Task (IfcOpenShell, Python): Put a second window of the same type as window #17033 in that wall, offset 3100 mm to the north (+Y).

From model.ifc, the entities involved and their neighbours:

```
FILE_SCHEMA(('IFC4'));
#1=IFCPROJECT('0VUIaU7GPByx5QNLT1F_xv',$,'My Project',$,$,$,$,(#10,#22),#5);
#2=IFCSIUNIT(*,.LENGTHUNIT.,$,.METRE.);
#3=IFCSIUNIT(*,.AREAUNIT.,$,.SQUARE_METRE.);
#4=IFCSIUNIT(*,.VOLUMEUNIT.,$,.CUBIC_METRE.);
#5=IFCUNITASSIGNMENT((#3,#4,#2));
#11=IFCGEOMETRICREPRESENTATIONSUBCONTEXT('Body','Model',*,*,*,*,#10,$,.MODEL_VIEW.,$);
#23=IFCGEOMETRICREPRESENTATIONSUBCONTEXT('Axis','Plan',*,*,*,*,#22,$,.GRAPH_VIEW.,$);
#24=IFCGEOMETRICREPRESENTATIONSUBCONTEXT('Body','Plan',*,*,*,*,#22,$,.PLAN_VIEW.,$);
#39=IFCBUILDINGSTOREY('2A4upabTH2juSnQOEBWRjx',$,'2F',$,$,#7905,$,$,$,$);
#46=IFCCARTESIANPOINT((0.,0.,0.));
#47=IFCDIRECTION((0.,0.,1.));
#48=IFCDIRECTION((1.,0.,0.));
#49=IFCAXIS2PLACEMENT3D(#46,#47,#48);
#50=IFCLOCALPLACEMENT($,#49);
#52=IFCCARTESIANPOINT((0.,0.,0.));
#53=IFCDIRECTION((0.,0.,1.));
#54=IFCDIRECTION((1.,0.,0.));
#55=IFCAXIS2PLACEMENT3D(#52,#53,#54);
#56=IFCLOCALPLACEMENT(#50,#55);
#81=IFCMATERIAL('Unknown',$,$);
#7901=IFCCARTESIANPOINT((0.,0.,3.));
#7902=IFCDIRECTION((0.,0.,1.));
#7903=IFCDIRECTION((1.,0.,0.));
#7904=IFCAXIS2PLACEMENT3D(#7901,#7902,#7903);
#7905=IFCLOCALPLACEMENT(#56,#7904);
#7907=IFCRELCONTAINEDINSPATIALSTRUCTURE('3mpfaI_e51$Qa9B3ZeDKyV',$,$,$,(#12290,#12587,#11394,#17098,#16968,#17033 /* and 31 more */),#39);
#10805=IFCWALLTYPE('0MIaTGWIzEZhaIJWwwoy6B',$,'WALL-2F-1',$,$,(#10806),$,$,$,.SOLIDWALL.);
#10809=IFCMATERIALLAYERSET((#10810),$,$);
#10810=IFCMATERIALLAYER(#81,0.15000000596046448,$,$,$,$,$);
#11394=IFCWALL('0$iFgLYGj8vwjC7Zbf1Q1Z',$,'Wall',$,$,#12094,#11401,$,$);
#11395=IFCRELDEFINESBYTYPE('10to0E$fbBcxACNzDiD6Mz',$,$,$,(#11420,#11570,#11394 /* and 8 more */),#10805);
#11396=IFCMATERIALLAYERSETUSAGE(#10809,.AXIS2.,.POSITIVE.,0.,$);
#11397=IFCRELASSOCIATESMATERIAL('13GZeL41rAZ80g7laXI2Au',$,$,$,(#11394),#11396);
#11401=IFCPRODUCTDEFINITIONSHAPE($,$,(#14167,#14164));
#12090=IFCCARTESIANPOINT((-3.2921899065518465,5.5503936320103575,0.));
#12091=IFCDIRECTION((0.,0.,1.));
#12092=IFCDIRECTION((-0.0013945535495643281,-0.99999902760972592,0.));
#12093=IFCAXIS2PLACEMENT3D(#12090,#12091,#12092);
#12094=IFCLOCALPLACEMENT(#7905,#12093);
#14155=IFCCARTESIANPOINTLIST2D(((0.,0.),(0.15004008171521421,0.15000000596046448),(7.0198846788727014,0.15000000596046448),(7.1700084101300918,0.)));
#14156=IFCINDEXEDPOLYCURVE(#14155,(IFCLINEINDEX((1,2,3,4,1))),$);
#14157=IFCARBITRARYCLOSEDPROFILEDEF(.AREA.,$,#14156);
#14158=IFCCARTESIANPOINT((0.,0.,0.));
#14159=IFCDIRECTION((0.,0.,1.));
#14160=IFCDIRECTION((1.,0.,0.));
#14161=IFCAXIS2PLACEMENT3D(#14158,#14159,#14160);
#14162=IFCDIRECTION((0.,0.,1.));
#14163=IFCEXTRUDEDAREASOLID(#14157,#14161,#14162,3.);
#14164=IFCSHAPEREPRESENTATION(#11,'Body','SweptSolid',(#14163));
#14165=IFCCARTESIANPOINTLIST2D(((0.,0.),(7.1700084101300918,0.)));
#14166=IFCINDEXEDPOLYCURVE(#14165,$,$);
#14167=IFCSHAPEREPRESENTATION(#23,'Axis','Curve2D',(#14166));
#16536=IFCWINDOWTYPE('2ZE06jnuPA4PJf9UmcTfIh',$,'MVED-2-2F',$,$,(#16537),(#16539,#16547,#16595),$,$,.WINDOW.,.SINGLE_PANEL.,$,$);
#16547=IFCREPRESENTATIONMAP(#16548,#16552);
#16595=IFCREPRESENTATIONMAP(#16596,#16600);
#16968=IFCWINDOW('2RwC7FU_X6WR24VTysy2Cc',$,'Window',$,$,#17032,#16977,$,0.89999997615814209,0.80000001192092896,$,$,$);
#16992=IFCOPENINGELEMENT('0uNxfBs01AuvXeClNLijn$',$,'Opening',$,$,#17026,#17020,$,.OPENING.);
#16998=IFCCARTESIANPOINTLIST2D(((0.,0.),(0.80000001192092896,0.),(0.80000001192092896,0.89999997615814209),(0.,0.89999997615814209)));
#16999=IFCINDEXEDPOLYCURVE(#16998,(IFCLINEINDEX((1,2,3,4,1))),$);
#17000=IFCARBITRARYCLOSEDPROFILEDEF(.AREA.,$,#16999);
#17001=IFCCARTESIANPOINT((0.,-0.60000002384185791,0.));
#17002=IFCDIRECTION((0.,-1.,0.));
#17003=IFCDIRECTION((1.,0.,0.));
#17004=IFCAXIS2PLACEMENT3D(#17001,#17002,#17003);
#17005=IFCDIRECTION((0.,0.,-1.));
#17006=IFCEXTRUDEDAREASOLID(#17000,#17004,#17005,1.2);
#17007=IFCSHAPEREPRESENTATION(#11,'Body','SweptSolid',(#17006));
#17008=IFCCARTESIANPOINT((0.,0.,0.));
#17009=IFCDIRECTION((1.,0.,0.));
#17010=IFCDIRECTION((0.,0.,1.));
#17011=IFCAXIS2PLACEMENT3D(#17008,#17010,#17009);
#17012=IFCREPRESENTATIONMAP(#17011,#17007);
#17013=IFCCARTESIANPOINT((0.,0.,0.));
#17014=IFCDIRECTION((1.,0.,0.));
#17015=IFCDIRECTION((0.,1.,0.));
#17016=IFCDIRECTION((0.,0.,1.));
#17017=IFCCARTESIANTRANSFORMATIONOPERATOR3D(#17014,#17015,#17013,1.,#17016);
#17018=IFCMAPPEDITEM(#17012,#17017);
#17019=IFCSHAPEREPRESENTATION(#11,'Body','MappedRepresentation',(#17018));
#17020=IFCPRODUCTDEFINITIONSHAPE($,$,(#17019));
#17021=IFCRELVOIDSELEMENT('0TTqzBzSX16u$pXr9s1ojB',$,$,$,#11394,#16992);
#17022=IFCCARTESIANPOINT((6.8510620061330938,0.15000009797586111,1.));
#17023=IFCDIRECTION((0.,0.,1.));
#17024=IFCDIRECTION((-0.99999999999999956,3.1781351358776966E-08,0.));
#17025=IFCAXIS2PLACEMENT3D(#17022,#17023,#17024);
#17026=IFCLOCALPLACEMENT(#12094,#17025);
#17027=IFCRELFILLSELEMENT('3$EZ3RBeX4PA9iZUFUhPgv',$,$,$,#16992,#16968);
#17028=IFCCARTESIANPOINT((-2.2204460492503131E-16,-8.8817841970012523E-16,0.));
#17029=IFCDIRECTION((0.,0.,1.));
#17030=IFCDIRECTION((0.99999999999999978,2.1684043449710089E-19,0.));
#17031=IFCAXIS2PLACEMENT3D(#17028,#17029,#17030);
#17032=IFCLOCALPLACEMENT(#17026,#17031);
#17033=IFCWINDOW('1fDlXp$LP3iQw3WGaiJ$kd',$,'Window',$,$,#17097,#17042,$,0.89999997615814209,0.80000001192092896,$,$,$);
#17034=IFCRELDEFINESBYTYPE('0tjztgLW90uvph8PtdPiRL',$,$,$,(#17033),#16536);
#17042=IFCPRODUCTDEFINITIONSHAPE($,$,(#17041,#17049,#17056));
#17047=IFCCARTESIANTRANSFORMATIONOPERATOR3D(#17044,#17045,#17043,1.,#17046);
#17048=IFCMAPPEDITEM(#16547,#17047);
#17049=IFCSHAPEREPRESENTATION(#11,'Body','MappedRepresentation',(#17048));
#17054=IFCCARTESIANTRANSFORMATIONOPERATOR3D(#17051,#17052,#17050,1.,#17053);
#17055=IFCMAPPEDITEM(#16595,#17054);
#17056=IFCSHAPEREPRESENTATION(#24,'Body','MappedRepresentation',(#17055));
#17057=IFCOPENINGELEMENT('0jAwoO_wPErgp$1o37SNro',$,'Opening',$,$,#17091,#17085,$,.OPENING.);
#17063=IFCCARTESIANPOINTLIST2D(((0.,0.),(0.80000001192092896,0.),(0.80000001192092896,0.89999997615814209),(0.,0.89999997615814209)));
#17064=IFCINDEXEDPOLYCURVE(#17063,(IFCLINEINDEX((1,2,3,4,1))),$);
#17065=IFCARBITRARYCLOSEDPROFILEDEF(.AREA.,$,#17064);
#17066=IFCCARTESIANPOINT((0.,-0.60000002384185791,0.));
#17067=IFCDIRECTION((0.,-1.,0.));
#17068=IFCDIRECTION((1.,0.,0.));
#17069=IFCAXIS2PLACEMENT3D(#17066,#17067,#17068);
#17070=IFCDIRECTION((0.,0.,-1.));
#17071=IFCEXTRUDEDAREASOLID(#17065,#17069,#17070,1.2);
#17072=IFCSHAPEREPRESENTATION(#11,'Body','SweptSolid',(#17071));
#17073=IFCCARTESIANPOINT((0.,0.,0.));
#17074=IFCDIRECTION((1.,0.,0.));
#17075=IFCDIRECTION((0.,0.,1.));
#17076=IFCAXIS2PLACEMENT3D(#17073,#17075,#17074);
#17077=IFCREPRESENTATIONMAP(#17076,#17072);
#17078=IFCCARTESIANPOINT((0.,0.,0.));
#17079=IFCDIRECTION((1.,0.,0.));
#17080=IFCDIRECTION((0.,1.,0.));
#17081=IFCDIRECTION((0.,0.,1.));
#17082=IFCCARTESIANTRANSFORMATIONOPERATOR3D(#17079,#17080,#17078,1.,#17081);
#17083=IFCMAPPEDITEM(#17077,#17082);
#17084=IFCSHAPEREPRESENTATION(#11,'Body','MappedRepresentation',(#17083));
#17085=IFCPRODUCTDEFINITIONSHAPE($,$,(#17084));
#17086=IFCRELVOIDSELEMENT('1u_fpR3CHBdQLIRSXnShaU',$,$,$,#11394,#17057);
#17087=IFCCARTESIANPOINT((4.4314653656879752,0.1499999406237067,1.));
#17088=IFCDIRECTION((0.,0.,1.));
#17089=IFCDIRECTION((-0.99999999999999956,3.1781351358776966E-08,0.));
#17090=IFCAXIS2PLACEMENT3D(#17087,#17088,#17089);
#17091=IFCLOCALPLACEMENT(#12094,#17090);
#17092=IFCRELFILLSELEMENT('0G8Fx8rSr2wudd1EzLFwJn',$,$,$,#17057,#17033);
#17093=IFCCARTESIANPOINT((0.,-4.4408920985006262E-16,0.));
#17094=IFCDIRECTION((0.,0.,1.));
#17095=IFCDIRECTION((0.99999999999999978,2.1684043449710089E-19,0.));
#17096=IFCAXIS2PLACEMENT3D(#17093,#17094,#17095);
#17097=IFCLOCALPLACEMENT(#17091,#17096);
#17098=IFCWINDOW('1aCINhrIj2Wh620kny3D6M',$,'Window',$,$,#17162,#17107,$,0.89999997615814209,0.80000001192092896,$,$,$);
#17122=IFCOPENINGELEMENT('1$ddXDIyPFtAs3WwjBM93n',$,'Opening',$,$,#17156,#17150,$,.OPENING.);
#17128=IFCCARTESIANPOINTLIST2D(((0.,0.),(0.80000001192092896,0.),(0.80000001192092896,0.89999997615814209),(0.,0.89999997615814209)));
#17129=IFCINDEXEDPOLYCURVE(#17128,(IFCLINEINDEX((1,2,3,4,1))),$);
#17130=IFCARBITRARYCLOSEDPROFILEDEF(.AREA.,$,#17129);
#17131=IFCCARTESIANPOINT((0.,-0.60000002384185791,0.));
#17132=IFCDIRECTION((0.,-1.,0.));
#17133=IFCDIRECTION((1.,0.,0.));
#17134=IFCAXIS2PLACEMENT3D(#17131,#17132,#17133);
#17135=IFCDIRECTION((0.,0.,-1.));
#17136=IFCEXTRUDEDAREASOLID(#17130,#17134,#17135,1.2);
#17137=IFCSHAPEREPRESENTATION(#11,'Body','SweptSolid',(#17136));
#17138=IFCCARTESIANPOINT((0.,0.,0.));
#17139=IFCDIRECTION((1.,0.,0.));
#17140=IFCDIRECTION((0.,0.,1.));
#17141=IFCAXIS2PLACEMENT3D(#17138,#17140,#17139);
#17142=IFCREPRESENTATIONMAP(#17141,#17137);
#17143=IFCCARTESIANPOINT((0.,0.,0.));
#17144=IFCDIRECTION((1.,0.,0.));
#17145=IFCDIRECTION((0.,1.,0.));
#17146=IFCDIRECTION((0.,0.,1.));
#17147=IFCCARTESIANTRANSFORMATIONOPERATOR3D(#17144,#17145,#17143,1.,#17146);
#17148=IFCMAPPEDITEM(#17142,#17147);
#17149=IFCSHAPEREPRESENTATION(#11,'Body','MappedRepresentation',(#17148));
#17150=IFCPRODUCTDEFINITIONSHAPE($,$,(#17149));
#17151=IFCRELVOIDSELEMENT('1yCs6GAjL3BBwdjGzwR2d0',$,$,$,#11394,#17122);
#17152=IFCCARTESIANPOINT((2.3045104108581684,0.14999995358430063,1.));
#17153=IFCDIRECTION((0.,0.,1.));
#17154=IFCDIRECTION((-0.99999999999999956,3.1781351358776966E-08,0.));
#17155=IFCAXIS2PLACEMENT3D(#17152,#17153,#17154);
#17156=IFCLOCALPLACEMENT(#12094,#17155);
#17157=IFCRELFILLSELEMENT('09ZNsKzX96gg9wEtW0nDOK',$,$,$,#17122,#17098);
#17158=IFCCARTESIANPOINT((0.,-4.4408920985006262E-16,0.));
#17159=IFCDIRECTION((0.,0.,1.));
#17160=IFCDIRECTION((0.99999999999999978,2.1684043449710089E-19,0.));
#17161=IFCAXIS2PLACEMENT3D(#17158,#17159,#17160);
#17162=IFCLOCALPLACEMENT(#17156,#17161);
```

```python
import ifcopenshell
import ifcopenshell.api.feature
import ifcopenshell.api.geometry
import ifcopenshell.api.root
import ifcopenshell.geom
import ifcopenshell.util.element
import ifcopenshell.util.placement
import ifcopenshell.util.shape
import ifcopenshell.util.unit

model = ifcopenshell.open("model.ifc")
unit_scale = ifcopenshell.util.unit.calculate_unit_scale(model)
settings = ifcopenshell.geom.settings()


def volume(element):
    """Net volume in cubic metres, openings subtracted."""
    shape = ifcopenshell.geom.create_shape(settings, element)
    return ifcopenshell.util.shape.get_volume(shape.geometry)


window = model.by_guid("1fDlXp$LP3iQw3WGaiJ$kd")
opening = window.FillsVoids[0].RelatingOpeningElement
wall = opening.VoidsElements[0].RelatingBuildingElement
before = volume(wall)
shift = ifcopenshell.util.placement.get_local_placement(wall.ObjectPlacement)[:3, 0] * -3.1 / unit_scale

# copy_class copies the void relationship, type, container and properties, but no geometry.
new_opening = ifcopenshell.api.root.copy_class(model, product=opening)
new_opening.Representation = ifcopenshell.util.element.copy_deep(
    model, opening.Representation, exclude=["IfcGeometricRepresentationContext", "IfcRepresentationMap"]
)
new_window = ifcopenshell.api.root.copy_class(model, product=window)
new_window.Representation = ifcopenshell.util.element.copy_deep(
    model, window.Representation, exclude=["IfcGeometricRepresentationContext", "IfcRepresentationMap"]
)
ifcopenshell.api.feature.add_filling(model, opening=new_opening, element=new_window)

for old, new in ((opening, new_opening), (window, new_window)):
    matrix = ifcopenshell.util.placement.get_local_placement(old.ObjectPlacement)
    matrix[:3, 3] += shift
    ifcopenshell.api.geometry.edit_object_placement(model, product=new, matrix=matrix, is_si=False)

after = volume(wall)

print(f"wall volume {before:.3f} -> {after:.3f} m3")

model.write("model-out.ifc")
```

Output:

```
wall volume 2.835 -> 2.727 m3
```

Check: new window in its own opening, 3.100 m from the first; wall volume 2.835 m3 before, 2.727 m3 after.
